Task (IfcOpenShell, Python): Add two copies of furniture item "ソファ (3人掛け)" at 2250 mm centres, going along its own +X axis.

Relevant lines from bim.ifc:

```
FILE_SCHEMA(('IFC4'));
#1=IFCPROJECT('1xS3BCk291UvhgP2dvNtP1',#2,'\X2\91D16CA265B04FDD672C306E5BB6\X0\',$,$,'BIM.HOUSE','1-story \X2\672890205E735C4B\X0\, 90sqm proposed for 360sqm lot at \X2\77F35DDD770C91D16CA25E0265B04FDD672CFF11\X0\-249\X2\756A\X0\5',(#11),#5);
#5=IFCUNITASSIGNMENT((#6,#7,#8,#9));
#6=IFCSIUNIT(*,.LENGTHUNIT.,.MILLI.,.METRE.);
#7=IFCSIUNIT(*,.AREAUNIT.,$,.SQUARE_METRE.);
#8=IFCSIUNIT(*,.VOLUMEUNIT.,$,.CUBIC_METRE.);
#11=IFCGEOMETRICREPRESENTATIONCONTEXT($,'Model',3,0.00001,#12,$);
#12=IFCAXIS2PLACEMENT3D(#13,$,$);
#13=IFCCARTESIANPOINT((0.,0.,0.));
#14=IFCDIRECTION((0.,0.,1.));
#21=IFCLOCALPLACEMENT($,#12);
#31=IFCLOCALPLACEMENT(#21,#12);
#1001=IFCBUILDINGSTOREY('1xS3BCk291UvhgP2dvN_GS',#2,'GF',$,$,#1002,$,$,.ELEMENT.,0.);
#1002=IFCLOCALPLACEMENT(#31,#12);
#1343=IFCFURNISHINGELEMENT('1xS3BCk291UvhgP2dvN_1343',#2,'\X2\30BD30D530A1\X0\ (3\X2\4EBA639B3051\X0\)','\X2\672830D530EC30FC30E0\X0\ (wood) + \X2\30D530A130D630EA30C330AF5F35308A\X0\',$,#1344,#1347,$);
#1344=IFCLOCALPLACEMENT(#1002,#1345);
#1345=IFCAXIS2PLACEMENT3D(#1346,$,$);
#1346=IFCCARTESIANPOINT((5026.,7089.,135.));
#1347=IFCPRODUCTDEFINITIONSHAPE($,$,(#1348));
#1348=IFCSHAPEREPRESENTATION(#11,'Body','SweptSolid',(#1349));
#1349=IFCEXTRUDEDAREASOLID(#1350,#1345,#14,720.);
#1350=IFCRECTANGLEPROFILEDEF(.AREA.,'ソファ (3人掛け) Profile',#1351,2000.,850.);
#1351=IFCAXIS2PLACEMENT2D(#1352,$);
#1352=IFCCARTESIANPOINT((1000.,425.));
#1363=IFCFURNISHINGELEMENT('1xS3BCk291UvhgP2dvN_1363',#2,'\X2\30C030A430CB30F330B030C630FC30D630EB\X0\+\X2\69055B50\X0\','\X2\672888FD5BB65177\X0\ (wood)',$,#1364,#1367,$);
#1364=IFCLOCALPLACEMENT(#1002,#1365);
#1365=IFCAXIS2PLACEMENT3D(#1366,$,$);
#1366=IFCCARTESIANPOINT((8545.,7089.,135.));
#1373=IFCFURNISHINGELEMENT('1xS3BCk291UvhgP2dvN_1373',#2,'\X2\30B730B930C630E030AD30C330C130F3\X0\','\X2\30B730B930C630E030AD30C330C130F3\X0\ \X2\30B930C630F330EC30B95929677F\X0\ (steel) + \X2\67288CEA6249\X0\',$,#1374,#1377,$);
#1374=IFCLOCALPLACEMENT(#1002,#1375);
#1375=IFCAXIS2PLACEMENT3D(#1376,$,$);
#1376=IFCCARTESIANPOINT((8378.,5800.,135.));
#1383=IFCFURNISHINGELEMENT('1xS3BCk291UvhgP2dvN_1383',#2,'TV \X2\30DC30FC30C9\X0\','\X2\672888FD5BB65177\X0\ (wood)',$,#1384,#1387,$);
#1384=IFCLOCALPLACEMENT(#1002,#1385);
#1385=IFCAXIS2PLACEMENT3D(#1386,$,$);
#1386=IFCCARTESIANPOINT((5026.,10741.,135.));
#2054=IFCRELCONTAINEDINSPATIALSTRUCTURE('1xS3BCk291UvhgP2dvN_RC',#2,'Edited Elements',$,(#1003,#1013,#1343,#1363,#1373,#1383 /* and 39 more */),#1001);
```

```python
import ifcopenshell
import ifcopenshell.api.geometry
import ifcopenshell.api.root
import ifcopenshell.util.element
import ifcopenshell.util.placement
import ifcopenshell.util.unit

model = ifcopenshell.open("bim.ifc")
unit_scale = ifcopenshell.util.unit.calculate_unit_scale(model)


def reuse_history(source, copy):
    """copy_class also copies each property set's owner history, people and application; keep the originals."""
    for rel in copy.IsDefinedBy:
        if rel.is_a("IfcRelDefinesByProperties") and (history := rel.RelatingPropertyDefinition.OwnerHistory):
            rel.RelatingPropertyDefinition.OwnerHistory = source.OwnerHistory
            ifcopenshell.util.element.remove_deep2(model, history)


source = model.by_guid("1xS3BCk291UvhgP2dvN_1343")
base = ifcopenshell.util.placement.get_local_placement(source.ObjectPlacement)
step = base[:3, 0] * 2.25 / unit_scale

for i in range(1, 3):
    copy = ifcopenshell.api.root.copy_class(model, product=source)
    copy.Representation = ifcopenshell.util.element.copy_deep(
        model, source.Representation, exclude=["IfcGeometricRepresentationContext", "IfcRepresentationMap"]
    )
    reuse_history(source, copy)
    matrix = base.copy()
    matrix[:3, 3] += i * step
    print("added at", matrix[:3, 3].round(3) + 0.0)
    ifcopenshell.api.geometry.edit_object_placement(model, product=copy, matrix=matrix, is_si=False)

model.write("bim_updated.ifc")
```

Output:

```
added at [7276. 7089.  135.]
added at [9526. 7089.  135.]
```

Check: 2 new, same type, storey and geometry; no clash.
